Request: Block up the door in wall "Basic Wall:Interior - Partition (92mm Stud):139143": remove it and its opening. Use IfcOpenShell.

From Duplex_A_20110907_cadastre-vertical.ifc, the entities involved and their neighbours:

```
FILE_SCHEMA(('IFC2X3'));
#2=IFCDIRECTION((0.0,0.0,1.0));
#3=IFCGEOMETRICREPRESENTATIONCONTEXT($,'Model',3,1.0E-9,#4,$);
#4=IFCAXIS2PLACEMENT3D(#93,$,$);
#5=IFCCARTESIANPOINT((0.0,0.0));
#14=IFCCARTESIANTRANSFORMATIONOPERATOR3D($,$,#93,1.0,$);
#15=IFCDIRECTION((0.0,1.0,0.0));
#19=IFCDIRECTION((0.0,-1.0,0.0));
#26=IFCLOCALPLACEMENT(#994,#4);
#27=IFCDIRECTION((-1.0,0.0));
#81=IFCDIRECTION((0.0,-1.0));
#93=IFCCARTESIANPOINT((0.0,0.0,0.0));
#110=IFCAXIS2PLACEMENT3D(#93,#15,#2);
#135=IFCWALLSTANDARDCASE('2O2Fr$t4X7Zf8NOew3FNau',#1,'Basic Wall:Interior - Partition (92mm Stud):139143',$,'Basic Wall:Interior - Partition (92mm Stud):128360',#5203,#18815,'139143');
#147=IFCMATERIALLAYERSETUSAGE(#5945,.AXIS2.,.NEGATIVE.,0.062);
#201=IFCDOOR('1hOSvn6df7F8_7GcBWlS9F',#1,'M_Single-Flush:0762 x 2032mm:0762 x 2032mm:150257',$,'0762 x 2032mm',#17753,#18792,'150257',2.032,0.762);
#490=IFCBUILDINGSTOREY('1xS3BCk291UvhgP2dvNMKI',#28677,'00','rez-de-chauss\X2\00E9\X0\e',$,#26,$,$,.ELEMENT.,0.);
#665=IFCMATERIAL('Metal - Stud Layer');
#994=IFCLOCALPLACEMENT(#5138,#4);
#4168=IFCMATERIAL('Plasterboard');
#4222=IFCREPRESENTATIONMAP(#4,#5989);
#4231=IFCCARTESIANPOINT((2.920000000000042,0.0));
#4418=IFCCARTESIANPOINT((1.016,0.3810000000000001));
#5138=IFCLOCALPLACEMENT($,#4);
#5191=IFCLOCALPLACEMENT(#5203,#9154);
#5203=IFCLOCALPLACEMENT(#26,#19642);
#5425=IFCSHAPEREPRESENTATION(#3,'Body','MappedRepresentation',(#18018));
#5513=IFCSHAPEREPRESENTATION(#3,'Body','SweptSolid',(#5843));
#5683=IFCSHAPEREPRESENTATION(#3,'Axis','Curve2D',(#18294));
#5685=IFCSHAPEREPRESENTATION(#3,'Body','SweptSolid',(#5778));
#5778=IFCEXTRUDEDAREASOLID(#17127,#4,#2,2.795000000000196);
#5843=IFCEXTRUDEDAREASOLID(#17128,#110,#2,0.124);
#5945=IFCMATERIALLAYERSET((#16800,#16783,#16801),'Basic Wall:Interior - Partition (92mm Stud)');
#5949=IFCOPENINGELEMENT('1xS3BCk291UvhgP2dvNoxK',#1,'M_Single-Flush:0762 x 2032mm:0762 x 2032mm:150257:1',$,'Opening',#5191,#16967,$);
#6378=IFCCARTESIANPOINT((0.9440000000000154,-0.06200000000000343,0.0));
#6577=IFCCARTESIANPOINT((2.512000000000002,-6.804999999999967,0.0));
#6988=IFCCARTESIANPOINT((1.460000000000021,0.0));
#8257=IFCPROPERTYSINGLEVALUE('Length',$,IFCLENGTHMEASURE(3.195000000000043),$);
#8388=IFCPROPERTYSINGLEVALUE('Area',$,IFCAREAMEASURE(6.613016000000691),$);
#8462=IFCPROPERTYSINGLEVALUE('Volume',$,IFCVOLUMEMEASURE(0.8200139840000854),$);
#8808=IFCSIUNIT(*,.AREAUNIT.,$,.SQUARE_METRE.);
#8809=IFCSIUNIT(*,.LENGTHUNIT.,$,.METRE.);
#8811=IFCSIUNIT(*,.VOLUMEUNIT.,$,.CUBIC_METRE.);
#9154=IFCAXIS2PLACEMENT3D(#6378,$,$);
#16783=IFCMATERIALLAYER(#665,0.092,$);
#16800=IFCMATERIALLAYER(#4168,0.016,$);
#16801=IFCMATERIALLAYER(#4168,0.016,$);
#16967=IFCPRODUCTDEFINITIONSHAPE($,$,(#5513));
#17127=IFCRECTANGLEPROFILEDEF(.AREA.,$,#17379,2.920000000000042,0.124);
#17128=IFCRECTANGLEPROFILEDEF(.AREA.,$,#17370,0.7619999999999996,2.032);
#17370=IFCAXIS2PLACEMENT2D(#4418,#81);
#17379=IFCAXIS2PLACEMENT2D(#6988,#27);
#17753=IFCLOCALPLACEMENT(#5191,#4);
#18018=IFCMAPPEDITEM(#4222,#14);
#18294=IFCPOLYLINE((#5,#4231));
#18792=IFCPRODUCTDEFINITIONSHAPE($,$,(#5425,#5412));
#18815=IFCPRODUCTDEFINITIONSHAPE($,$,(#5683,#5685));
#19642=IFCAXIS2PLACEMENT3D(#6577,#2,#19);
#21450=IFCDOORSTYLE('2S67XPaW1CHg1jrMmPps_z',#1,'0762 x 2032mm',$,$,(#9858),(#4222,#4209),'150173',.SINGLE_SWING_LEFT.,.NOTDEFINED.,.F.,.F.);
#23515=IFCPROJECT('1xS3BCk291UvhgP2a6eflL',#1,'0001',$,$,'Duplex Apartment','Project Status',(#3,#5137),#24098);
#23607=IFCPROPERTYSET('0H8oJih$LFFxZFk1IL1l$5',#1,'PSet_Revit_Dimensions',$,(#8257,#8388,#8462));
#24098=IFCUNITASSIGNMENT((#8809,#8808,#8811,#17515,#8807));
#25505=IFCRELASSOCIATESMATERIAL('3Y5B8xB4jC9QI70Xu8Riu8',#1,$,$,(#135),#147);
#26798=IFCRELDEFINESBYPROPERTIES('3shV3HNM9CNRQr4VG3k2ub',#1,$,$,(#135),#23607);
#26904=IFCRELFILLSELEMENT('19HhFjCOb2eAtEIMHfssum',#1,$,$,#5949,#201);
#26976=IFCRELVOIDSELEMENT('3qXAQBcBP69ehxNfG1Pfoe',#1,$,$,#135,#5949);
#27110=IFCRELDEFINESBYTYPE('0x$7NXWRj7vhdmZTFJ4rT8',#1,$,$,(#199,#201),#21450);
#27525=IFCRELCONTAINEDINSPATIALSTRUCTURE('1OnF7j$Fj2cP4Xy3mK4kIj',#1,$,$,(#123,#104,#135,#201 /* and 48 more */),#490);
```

```python
import ifcopenshell
import ifcopenshell.api.feature
import ifcopenshell.api.pset
import ifcopenshell.api.root
import ifcopenshell.geom
import ifcopenshell.util.element
import ifcopenshell.util.shape
import ifcopenshell.util.unit

model = ifcopenshell.open("Duplex_A_20110907_cadastre-vertical.ifc")
area_scale = ifcopenshell.util.unit.calculate_unit_scale(model, "AREAUNIT")
volume_scale = ifcopenshell.util.unit.calculate_unit_scale(model, "VOLUMEUNIT")
settings = ifcopenshell.geom.settings()


def volume(element):
    """Net volume in cubic metres, openings subtracted."""
    shape = ifcopenshell.geom.create_shape(settings, element)
    return ifcopenshell.util.shape.get_volume(shape.geometry)


door = model.by_guid("1hOSvn6df7F8_7GcBWlS9F")
opening = door.FillsVoids[0].RelatingOpeningElement
wall = opening.VoidsElements[0].RelatingBuildingElement
before = volume(wall)

ifcopenshell.api.root.remove_product(model, product=door)
ifcopenshell.api.feature.remove_feature(model, feature=opening)

after = volume(wall)
thickness = 0.124  # wall thickness in metres

# Update the wall's stored quantities.
pset = model.by_id(ifcopenshell.util.element.get_pset(wall, "PSet_Revit_Dimensions", should_inherit=False)["id"])
ifcopenshell.api.pset.edit_pset(model, pset=pset, properties={
    "Area": model.create_entity("IfcAreaMeasure", after / thickness / area_scale),
    "Volume": model.create_entity("IfcVolumeMeasure", after / volume_scale),
})

print(f"wall volume {before:.3f} -> {after:.3f} m3")

model.write("Duplex_A_20110907_cadastre-vertical-out.ifc")
```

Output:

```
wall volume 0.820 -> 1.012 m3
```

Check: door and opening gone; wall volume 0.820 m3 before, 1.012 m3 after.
